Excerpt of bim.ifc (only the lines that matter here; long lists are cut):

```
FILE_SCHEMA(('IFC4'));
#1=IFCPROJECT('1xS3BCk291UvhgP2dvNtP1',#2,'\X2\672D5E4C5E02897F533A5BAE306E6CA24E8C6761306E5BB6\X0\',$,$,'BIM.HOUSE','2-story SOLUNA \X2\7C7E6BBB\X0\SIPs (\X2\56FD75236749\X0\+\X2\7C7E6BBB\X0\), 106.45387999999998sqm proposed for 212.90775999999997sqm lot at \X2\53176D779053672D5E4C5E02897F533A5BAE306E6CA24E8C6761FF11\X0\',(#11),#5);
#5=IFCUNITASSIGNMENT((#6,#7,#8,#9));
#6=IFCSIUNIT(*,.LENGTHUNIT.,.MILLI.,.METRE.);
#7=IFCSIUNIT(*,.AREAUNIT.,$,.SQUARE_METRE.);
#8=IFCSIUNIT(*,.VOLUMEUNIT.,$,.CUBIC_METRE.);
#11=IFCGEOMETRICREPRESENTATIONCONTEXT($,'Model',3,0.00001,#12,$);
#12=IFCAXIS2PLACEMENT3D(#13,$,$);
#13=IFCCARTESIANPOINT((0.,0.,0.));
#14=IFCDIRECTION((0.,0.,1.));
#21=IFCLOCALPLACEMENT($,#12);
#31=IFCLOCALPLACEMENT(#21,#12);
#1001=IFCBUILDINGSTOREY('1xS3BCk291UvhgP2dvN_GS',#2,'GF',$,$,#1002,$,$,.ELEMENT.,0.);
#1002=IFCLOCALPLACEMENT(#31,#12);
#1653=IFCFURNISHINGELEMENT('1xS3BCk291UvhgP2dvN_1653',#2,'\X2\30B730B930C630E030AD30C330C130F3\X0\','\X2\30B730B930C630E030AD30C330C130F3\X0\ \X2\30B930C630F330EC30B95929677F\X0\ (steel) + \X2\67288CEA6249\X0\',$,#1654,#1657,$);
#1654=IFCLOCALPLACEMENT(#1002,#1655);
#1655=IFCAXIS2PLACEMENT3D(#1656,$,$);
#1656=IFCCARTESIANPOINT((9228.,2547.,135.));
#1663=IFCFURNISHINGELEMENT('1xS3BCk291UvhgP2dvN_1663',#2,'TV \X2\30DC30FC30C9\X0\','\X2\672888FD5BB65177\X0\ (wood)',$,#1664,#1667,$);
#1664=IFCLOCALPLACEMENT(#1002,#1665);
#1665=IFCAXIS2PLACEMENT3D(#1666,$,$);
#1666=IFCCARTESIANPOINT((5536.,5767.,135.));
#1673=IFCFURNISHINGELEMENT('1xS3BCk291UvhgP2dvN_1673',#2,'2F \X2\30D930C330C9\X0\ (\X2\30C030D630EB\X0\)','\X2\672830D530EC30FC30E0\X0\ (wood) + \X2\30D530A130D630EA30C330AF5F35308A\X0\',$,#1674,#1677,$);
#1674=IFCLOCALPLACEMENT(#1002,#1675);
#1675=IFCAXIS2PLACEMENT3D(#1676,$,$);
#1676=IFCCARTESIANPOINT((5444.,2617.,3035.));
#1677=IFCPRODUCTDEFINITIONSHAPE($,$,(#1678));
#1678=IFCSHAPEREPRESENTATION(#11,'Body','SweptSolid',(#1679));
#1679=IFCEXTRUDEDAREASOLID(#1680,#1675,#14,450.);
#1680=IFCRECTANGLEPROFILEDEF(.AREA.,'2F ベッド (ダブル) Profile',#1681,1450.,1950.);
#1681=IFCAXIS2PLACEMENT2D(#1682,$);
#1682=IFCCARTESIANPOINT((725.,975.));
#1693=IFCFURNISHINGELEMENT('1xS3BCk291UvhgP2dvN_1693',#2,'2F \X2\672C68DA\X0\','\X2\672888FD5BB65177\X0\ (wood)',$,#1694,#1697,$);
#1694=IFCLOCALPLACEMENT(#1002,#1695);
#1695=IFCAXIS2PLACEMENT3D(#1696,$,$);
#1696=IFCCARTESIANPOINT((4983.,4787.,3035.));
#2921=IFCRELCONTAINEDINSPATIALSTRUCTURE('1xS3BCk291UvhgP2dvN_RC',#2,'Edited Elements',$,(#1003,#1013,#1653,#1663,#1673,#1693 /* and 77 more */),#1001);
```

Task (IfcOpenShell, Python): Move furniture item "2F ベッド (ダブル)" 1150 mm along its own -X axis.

```python
import ifcopenshell
import ifcopenshell.api.geometry
import ifcopenshell.util.placement

model = ifcopenshell.open("bim.ifc")

item = model.by_id(1673)
matrix = ifcopenshell.util.placement.get_local_placement(item.ObjectPlacement)
matrix[:3, 3] -= matrix[:3, 0] * 1150.0
ifcopenshell.api.geometry.edit_object_placement(model, product=item, matrix=matrix, is_si=False)

print(ifcopenshell.util.placement.get_local_placement(item.ObjectPlacement).round(3) + 0.0)

model.write("bim_v2.ifc")
```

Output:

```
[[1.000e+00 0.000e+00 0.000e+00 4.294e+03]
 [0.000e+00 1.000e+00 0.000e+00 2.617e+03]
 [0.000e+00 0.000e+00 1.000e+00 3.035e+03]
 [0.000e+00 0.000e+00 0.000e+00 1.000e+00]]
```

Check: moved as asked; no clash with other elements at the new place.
